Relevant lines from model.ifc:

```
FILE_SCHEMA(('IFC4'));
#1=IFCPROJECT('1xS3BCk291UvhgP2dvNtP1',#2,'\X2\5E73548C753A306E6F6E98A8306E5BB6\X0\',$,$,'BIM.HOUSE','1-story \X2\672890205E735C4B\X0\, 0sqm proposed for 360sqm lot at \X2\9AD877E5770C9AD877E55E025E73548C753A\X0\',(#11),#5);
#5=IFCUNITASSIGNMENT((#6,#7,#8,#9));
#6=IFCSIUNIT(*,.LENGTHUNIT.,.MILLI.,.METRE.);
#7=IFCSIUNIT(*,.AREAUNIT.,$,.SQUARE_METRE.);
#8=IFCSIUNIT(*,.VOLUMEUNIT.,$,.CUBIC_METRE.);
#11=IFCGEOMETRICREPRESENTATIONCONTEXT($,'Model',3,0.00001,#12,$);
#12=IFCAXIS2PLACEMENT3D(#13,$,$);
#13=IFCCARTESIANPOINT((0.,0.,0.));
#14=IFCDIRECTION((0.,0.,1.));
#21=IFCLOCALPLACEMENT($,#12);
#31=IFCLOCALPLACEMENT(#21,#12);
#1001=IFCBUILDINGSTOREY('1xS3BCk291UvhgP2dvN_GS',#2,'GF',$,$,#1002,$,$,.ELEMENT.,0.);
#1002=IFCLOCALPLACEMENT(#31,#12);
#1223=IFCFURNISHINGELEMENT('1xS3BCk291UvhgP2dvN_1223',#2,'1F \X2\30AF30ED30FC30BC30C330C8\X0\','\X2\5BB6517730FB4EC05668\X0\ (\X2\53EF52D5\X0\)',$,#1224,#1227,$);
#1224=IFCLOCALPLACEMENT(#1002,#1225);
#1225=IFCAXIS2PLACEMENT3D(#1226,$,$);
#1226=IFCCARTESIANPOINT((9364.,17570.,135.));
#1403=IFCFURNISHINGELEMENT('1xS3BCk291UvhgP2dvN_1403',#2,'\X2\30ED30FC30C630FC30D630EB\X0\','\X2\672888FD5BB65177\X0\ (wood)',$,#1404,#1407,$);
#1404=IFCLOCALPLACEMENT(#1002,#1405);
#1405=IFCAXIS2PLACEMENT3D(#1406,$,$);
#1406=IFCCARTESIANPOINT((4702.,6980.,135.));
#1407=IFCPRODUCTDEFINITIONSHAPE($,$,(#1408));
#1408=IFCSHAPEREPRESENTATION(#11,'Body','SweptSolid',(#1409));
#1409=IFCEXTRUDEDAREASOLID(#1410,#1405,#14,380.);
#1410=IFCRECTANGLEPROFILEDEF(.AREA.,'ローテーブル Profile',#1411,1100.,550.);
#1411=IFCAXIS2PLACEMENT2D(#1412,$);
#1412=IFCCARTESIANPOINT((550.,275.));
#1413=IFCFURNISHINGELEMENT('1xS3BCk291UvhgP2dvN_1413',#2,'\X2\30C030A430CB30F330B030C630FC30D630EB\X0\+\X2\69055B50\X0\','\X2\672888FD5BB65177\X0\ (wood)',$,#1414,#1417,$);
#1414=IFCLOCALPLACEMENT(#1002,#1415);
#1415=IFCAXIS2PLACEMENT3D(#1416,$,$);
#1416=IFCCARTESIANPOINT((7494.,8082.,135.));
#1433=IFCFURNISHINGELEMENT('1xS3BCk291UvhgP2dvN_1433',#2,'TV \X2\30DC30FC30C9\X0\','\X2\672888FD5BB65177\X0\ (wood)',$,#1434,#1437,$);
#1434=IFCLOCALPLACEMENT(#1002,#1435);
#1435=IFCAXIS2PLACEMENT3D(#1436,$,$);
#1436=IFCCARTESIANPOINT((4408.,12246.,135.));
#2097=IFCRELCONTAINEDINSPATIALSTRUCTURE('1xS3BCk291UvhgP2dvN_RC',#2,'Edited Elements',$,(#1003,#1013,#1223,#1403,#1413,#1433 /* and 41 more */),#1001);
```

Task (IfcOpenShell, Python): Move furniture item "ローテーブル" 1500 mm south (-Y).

```python
import ifcopenshell
import ifcopenshell.api.geometry
import ifcopenshell.util.placement
import ifcopenshell.util.unit

model = ifcopenshell.open("model.ifc")
unit_scale = ifcopenshell.util.unit.calculate_unit_scale(model)

item = model.by_guid("1xS3BCk291UvhgP2dvN_1403")
matrix = ifcopenshell.util.placement.get_local_placement(item.ObjectPlacement)
matrix[1, 3] -= 1.5 / unit_scale
ifcopenshell.api.geometry.edit_object_placement(model, product=item, matrix=matrix, is_si=False)

print(ifcopenshell.util.placement.get_local_placement(item.ObjectPlacement).round(3) + 0.0)

model.write("model-out.ifc")
```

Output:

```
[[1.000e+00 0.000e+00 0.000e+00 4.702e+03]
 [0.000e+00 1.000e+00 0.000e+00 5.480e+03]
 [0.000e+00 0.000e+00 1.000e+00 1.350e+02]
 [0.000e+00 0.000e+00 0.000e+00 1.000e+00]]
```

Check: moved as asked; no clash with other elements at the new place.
